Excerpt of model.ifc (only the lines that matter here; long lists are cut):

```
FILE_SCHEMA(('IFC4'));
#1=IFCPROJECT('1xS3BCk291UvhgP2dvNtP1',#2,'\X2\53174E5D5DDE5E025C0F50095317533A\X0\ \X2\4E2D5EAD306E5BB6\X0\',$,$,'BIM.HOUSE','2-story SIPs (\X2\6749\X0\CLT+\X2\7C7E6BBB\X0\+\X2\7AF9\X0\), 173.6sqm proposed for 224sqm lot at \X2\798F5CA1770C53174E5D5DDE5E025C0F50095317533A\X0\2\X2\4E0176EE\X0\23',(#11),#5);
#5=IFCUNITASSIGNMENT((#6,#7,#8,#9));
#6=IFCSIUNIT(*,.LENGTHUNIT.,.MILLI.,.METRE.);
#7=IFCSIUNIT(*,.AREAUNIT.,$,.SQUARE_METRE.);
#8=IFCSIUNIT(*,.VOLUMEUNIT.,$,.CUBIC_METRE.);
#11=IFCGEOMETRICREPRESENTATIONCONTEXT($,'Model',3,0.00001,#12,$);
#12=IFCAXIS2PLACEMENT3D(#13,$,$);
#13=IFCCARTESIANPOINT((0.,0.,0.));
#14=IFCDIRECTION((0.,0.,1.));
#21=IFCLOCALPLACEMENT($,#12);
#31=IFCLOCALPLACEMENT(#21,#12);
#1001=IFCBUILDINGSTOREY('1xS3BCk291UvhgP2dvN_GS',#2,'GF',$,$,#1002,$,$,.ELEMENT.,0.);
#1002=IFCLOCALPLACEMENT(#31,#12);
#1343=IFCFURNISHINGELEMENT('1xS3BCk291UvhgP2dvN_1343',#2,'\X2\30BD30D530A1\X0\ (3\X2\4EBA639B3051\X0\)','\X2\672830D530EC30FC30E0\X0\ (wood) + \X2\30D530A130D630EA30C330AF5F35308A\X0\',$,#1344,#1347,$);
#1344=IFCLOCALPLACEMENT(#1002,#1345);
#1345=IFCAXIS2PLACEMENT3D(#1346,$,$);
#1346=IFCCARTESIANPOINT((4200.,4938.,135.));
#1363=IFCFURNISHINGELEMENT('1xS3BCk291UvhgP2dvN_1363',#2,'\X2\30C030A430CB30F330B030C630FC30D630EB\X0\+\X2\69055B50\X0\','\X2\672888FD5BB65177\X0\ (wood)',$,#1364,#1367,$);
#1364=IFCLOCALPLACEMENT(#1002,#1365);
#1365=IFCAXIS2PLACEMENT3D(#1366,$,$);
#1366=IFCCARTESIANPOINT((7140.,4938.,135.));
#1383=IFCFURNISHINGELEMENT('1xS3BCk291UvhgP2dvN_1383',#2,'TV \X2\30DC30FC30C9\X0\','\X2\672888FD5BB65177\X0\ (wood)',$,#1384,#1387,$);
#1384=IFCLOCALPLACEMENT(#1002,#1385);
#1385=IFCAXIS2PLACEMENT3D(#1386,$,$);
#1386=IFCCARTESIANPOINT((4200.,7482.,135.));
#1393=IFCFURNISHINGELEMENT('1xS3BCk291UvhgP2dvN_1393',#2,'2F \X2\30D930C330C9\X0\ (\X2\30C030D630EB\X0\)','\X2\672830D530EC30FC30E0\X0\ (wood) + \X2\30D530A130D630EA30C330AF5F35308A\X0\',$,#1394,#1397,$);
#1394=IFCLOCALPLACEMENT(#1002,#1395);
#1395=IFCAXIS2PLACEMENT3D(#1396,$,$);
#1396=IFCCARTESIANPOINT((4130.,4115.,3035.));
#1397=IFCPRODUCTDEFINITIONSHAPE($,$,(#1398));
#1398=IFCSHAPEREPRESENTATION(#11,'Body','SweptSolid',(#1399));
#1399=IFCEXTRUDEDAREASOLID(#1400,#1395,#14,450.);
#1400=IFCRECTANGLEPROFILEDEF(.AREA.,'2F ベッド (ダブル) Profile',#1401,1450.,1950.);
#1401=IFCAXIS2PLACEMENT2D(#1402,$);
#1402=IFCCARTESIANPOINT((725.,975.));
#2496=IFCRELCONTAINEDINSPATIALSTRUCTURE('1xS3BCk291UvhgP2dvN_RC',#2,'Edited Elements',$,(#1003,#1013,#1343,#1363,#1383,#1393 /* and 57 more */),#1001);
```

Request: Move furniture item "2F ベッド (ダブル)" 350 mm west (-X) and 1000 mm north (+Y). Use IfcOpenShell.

```python
import ifcopenshell
import ifcopenshell.api.geometry
import ifcopenshell.util.placement

model = ifcopenshell.open("model.ifc")

item = model.by_guid("1xS3BCk291UvhgP2dvN_1393")
matrix = ifcopenshell.util.placement.get_local_placement(item.ObjectPlacement)
matrix[0, 3] -= 350.0
matrix[1, 3] += 1000.0
ifcopenshell.api.geometry.edit_object_placement(model, product=item, matrix=matrix, is_si=False)

print(ifcopenshell.util.placement.get_local_placement(item.ObjectPlacement).round(3) + 0.0)

model.write("model_rev.ifc")
```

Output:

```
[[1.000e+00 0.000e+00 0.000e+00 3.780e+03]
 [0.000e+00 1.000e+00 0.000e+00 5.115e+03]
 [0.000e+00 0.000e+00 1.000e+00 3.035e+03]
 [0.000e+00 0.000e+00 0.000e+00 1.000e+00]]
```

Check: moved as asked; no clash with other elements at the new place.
